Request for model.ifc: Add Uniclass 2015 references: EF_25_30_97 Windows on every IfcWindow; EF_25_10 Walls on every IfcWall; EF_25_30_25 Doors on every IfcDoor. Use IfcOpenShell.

First a look at what the model holds.

```python
import ifcopenshell

model = ifcopenshell.open("model.ifc")
print(model.schema)
print("classifications:", [c.Name for c in model.by_type("IfcClassification")])
for ifc_class in ("IfcDoor", "IfcRoof", "IfcStair", "IfcWall", "IfcWindow"):
    print(ifc_class, len(model.by_type(ifc_class)))
```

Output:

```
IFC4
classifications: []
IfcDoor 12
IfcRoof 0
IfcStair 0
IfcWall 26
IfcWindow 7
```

```python
import ifcopenshell
import ifcopenshell.api.classification

model = ifcopenshell.open("model.ifc")

system = ifcopenshell.api.classification.add_classification(model, classification="Uniclass 2015")

codes = {
    "IfcWindow": ("EF_25_30_97", "Windows"),
    "IfcWall": ("EF_25_10", "Walls"),
    "IfcDoor": ("EF_25_30_25", "Doors"),
}
for ifc_class, (code, name) in codes.items():
    products = model.by_type(ifc_class)
    ifcopenshell.api.classification.add_reference(
        model, products=products, classification=system, identification=code, name=name
    )
    print(code, len(products))

model.write("model_v2.ifc")
```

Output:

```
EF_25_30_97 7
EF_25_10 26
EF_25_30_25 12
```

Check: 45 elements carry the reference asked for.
